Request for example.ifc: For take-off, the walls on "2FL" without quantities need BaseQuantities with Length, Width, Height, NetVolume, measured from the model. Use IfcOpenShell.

First a look at what the model holds.

```python
import ifcopenshell
import ifcopenshell.util.element
import ifcopenshell.util.unit

model = ifcopenshell.open("example.ifc")
print(model.schema)
for unit_type in ("LENGTHUNIT", "AREAUNIT", "VOLUMEUNIT"):
    print(unit_type, ifcopenshell.util.unit.calculate_unit_scale(model, unit_type))
storey = next(s for s in model.by_type("IfcBuildingStorey") if s.Name == "2FL")
walls = [e for e in ifcopenshell.util.element.get_decomposition(storey) if e.is_a("IfcWall")]
for e in sorted(walls, key=lambda e: e.id()):
    print(e.id(), e.is_a(), e.Name, list(ifcopenshell.util.element.get_psets(e, qtos_only=True)), sep=" | ")
```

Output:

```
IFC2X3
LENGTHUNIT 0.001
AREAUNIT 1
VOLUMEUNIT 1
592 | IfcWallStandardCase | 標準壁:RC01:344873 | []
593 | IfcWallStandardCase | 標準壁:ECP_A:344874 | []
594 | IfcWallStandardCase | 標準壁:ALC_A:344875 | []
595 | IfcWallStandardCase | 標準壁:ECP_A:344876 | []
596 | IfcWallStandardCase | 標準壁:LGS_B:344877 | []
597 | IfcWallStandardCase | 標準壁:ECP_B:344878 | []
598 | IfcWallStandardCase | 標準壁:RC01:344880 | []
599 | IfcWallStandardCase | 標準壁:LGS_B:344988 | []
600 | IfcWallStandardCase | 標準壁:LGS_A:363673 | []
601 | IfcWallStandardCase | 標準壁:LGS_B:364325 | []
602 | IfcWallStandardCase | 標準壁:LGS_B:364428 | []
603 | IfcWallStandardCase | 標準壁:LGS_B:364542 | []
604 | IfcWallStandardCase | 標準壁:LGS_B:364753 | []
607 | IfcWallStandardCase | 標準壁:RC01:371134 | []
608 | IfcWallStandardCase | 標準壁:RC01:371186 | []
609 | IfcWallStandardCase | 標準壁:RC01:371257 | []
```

```python
import ifcopenshell
import ifcopenshell.api.pset
import ifcopenshell.geom
import ifcopenshell.util.element
import ifcopenshell.util.shape
import ifcopenshell.util.unit

model = ifcopenshell.open("example.ifc")
unit_scale = ifcopenshell.util.unit.calculate_unit_scale(model)
volume_scale = ifcopenshell.util.unit.calculate_unit_scale(model, "VOLUMEUNIT")
settings = ifcopenshell.geom.settings()

storey = next(s for s in model.by_type("IfcBuildingStorey") if s.Name == "2FL")
walls = [e for e in ifcopenshell.util.element.get_decomposition(storey) if e.is_a("IfcWall")]

for e in sorted(walls, key=lambda e: e.id()):
    if ifcopenshell.util.element.get_psets(e, qtos_only=True, should_inherit=False):
        continue
    # Geometry comes back in metres, in the element's own axes.
    shape = ifcopenshell.geom.create_shape(settings, e)
    values = {
        "Length": ifcopenshell.util.shape.get_x(shape.geometry) / unit_scale,
        "Width": ifcopenshell.util.shape.get_y(shape.geometry) / unit_scale,
        "Height": ifcopenshell.util.shape.get_z(shape.geometry) / unit_scale,
        "NetVolume": ifcopenshell.util.shape.get_volume(shape.geometry) / volume_scale,
    }
    qto = ifcopenshell.api.pset.add_qto(model, product=e, name="BaseQuantities")
    ifcopenshell.api.pset.edit_qto(model, qto=qto, properties=values)
    print(e.id(), {k: round(v, 3) for k, v in values.items()})

model.write("example-out.ifc")
```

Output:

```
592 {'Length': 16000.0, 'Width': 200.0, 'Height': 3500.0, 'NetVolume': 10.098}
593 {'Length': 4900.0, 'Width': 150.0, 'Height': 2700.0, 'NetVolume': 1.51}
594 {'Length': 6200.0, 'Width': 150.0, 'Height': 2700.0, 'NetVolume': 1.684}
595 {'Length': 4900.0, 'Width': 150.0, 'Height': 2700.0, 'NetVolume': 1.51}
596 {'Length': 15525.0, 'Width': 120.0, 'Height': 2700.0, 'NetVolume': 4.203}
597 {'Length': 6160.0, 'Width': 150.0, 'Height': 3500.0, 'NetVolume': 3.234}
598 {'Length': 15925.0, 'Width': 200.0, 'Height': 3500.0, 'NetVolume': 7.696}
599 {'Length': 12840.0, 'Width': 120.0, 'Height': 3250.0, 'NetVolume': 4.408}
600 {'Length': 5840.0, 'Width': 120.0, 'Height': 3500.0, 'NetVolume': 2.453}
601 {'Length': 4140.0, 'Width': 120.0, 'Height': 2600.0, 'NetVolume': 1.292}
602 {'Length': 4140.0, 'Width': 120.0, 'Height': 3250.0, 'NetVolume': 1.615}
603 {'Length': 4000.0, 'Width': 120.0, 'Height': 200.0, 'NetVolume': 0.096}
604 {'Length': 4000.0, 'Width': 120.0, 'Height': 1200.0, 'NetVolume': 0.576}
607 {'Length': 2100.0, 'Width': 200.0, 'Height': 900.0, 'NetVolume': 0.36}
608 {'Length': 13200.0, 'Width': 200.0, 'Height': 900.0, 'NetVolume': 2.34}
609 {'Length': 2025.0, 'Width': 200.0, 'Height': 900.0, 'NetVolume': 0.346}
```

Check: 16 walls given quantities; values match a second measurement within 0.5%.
